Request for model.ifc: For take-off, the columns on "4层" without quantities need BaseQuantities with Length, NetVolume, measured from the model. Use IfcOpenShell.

First a look at what the model holds.

```python
import ifcopenshell
import ifcopenshell.util.element
import ifcopenshell.util.unit

model = ifcopenshell.open("model.ifc")
print(model.schema)
for unit_type in ("LENGTHUNIT", "AREAUNIT", "VOLUMEUNIT"):
    print(unit_type, ifcopenshell.util.unit.calculate_unit_scale(model, unit_type))
storey = next(s for s in model.by_type("IfcBuildingStorey") if s.Name == "4层")
columns = [e for e in ifcopenshell.util.element.get_decomposition(storey) if e.is_a("IfcColumn")]
for e in sorted(columns, key=lambda e: e.id()):
    print(e.id(), e.is_a(), e.Name, list(ifcopenshell.util.element.get_psets(e, qtos_only=True)), sep=" | ")
```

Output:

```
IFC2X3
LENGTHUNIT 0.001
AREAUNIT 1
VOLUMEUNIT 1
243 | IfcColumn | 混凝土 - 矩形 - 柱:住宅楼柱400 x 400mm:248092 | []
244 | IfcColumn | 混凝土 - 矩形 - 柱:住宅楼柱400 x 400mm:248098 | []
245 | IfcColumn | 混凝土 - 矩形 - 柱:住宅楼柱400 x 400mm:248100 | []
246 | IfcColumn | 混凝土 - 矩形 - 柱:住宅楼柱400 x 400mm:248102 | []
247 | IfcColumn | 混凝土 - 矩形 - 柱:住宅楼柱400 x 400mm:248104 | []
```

```python
import ifcopenshell
import ifcopenshell.api.pset
import ifcopenshell.geom
import ifcopenshell.util.element
import ifcopenshell.util.shape
import ifcopenshell.util.unit

model = ifcopenshell.open("model.ifc")
unit_scale = ifcopenshell.util.unit.calculate_unit_scale(model)
volume_scale = ifcopenshell.util.unit.calculate_unit_scale(model, "VOLUMEUNIT")
settings = ifcopenshell.geom.settings()

storey = next(s for s in model.by_type("IfcBuildingStorey") if s.Name == "4层")
columns = [e for e in ifcopenshell.util.element.get_decomposition(storey) if e.is_a("IfcColumn")]

for e in sorted(columns, key=lambda e: e.id()):
    if ifcopenshell.util.element.get_psets(e, qtos_only=True, should_inherit=False):
        continue
    # Geometry comes back in metres, in the element's own axes.
    shape = ifcopenshell.geom.create_shape(settings, e)
    values = {
        "Length": ifcopenshell.util.shape.get_z(shape.geometry) / unit_scale,
        "NetVolume": ifcopenshell.util.shape.get_volume(shape.geometry) / volume_scale,
    }
    qto = ifcopenshell.api.pset.add_qto(model, product=e, name="BaseQuantities")
    ifcopenshell.api.pset.edit_qto(model, qto=qto, properties=values)
    print(e.id(), {k: round(v, 3) for k, v in values.items()})

model.write("model_updated.ifc")
```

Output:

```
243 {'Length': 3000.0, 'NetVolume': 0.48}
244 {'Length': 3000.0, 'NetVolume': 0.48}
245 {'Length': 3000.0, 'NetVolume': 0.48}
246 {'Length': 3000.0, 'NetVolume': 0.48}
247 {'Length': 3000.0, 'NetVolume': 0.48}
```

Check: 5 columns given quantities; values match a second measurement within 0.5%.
